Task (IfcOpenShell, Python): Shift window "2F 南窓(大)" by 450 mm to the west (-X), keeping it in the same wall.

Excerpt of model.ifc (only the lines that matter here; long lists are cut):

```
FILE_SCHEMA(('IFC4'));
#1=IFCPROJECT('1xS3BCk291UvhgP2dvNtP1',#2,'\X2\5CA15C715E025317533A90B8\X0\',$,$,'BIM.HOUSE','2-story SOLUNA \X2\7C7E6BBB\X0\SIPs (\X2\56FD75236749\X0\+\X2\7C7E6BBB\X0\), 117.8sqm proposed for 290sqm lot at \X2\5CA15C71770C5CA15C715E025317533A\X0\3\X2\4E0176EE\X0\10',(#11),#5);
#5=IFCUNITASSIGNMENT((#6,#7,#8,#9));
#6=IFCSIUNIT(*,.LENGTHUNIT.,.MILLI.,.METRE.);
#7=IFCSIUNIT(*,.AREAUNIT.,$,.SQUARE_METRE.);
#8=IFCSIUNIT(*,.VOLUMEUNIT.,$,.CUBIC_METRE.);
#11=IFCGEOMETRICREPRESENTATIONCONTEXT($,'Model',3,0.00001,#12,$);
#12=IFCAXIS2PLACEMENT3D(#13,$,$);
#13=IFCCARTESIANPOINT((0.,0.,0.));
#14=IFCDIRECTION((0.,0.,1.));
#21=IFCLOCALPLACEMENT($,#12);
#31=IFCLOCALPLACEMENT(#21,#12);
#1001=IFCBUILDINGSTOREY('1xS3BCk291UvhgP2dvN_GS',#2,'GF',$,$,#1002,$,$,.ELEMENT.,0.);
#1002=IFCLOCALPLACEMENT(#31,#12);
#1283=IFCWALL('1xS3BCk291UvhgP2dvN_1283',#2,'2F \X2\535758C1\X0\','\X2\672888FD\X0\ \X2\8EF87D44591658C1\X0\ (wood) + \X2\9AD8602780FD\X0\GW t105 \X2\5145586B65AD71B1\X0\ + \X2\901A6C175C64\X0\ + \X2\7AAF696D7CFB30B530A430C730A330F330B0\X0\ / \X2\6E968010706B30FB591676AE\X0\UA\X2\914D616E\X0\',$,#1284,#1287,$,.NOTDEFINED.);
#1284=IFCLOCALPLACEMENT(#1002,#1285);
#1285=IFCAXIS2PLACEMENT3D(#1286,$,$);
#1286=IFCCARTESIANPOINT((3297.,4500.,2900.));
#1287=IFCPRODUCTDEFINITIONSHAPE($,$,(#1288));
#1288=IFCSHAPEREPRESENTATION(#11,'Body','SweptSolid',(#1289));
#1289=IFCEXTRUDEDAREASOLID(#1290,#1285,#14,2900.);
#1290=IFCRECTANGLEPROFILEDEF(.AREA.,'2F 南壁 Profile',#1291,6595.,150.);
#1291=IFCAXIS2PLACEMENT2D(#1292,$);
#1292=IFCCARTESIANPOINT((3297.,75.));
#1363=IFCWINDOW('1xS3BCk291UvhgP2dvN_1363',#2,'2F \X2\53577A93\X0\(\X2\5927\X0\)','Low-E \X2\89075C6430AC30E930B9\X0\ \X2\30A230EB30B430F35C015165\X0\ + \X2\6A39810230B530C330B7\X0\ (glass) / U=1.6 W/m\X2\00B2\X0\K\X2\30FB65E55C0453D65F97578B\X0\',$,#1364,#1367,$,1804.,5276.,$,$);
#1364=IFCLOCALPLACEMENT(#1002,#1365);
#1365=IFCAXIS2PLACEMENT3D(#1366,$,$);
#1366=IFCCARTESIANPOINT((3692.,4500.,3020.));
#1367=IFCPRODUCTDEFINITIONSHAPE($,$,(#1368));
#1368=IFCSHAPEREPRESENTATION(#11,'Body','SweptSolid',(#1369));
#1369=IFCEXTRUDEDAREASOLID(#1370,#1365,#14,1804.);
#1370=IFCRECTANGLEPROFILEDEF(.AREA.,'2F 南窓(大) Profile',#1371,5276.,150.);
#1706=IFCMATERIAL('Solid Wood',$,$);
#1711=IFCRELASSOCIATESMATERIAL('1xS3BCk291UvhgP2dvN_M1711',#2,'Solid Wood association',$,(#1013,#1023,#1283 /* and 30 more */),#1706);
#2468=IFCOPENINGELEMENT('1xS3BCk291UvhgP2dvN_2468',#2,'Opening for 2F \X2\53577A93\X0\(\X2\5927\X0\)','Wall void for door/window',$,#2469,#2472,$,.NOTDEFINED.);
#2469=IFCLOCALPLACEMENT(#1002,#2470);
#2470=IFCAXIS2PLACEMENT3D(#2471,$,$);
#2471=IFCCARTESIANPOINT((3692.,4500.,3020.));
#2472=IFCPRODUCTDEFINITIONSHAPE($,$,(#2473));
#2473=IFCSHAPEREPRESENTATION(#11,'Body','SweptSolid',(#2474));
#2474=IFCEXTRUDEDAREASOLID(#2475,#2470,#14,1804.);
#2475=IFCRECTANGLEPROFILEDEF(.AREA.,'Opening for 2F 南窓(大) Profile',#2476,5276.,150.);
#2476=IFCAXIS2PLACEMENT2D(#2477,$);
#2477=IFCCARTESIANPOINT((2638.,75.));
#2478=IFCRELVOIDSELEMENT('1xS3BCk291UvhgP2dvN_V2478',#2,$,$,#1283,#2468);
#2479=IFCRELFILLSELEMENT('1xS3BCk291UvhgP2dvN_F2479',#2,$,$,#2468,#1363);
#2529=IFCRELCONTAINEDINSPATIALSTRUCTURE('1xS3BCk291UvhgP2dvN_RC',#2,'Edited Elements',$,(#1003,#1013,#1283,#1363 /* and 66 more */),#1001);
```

```python
import ifcopenshell
import ifcopenshell.api.geometry
import ifcopenshell.util.placement
import ifcopenshell.util.unit

model = ifcopenshell.open("model.ifc")
unit_scale = ifcopenshell.util.unit.calculate_unit_scale(model)

window = model.by_guid("1xS3BCk291UvhgP2dvN_1363")
opening = window.FillsVoids[0].RelatingOpeningElement
wall = opening.VoidsElements[0].RelatingBuildingElement

wall_matrix = ifcopenshell.util.placement.get_local_placement(wall.ObjectPlacement)
shift = wall_matrix[:3, 0] * -0.45 / unit_scale
before = ifcopenshell.util.placement.get_local_placement(window.ObjectPlacement)[:3, 3].copy()

# The window is not placed relative to its opening, so move both.
for product in (opening, window):
    matrix = ifcopenshell.util.placement.get_local_placement(product.ObjectPlacement)
    matrix[:3, 3] += shift
    ifcopenshell.api.geometry.edit_object_placement(model, product=product, matrix=matrix, is_si=False)

after = ifcopenshell.util.placement.get_local_placement(window.ObjectPlacement)[:3, 3]
print("window moved by", (after - before).round(3) + 0.0)

model.write("model-out.ifc")
```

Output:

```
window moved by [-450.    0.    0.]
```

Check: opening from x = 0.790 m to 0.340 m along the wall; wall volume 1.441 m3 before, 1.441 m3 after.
